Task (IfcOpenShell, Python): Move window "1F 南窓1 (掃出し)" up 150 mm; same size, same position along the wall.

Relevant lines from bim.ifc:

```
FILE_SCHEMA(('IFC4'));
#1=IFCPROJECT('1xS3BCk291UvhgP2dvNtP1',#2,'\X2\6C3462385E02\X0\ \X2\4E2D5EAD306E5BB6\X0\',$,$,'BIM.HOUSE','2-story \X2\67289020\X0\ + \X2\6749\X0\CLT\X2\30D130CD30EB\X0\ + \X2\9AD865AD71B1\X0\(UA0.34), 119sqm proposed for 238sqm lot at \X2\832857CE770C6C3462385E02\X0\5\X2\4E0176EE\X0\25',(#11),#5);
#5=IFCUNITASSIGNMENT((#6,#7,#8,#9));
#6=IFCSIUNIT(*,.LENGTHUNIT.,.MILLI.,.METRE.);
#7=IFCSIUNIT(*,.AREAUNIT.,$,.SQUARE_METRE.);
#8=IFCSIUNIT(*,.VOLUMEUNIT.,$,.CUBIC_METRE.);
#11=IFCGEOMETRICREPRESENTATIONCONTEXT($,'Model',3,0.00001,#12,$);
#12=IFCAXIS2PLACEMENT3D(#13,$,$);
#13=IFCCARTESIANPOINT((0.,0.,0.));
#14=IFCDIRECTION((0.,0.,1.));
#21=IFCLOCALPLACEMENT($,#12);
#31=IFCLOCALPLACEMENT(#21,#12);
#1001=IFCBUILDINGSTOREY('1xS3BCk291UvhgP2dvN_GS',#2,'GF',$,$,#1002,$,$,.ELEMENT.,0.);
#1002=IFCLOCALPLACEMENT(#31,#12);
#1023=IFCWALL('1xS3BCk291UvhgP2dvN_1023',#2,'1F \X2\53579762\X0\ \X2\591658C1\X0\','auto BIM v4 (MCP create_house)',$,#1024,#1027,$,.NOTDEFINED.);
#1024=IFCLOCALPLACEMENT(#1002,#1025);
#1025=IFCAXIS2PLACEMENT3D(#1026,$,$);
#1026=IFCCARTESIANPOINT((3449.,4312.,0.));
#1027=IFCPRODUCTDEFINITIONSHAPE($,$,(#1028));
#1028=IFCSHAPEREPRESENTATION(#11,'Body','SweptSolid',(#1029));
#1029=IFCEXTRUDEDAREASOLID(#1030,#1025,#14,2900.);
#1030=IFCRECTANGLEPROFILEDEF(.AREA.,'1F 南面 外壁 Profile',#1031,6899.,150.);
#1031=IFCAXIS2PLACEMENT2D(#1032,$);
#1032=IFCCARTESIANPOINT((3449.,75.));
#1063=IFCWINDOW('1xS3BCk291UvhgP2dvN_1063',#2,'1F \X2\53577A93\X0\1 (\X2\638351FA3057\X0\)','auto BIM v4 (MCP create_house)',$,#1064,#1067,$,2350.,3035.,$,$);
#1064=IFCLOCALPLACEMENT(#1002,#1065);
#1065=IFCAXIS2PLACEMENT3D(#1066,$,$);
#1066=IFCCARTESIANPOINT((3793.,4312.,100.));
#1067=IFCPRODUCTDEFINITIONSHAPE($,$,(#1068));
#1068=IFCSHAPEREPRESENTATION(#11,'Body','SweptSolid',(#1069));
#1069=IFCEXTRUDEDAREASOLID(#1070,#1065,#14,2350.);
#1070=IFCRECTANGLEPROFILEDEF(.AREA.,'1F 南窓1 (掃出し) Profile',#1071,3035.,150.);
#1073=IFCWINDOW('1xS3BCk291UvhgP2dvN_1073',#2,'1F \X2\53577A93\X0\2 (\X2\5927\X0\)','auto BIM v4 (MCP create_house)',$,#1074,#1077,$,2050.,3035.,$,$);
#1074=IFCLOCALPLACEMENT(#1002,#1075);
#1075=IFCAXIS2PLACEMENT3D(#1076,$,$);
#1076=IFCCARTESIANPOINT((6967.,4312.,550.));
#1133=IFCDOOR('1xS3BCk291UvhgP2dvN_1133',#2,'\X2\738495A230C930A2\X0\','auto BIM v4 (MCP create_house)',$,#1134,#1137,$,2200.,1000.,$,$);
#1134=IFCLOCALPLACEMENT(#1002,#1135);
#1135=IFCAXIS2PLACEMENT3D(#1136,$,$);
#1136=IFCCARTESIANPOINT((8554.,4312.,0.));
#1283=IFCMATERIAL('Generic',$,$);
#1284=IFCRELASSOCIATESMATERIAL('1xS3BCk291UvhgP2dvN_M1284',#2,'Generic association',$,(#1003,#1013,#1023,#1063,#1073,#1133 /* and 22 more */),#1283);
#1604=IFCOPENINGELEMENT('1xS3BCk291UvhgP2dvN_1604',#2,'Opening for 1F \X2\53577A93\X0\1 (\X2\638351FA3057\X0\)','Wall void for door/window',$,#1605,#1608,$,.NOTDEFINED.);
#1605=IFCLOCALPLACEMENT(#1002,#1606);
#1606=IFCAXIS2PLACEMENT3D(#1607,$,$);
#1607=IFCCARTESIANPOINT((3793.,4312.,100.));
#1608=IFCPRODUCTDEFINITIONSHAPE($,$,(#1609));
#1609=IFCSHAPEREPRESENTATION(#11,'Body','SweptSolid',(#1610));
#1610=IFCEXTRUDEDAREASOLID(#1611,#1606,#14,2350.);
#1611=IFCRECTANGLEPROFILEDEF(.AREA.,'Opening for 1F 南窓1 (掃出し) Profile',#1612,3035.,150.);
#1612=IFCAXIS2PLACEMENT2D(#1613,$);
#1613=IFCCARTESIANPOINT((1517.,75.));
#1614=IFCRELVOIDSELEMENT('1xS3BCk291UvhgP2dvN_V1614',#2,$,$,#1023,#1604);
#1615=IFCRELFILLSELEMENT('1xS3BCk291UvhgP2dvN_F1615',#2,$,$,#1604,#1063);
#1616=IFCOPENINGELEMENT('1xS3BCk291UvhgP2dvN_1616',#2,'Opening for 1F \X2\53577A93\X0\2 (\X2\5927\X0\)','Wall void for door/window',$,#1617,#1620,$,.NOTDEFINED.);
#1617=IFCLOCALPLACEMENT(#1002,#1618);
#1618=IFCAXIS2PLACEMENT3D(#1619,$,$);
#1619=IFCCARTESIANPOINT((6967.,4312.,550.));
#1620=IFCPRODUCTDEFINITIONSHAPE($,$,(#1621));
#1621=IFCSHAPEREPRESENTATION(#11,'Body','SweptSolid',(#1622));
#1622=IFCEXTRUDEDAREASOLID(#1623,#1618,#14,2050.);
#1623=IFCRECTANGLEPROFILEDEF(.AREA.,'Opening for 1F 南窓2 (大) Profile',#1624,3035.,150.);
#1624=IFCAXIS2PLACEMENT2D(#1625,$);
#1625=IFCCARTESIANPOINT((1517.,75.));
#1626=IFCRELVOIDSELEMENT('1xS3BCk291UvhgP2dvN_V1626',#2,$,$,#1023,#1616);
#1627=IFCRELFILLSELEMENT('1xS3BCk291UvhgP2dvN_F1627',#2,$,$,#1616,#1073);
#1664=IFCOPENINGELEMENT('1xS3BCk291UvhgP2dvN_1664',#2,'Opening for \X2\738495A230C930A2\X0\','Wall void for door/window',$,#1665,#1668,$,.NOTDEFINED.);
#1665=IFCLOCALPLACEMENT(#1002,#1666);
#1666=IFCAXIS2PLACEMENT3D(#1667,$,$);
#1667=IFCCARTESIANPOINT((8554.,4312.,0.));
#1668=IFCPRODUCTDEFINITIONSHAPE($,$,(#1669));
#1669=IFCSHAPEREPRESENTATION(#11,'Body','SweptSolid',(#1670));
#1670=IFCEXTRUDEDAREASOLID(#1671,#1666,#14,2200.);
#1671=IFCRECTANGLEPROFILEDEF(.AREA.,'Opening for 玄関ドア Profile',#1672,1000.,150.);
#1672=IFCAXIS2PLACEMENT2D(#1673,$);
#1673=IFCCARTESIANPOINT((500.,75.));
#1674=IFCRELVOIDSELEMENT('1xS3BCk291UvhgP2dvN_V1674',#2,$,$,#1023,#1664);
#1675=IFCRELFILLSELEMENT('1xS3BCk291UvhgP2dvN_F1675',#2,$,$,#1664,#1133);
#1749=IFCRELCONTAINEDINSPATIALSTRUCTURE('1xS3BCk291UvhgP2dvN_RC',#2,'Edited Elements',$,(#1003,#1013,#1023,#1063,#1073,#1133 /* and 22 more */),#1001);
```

```python
import numpy as np
import ifcopenshell
import ifcopenshell.api.geometry
import ifcopenshell.util.placement
import ifcopenshell.util.unit

model = ifcopenshell.open("bim.ifc")
unit_scale = ifcopenshell.util.unit.calculate_unit_scale(model)

window = model.by_guid("1xS3BCk291UvhgP2dvN_1063")
opening = window.FillsVoids[0].RelatingOpeningElement
dz = 0.15 / unit_scale

shift = np.array([0.0, 0.0, dz])
# The window is not placed relative to its opening, so move both.
for product in (opening, window):
    matrix = ifcopenshell.util.placement.get_local_placement(product.ObjectPlacement)
    matrix[:3, 3] += shift
    ifcopenshell.api.geometry.edit_object_placement(model, product=product, matrix=matrix, is_si=False)

print(f"moved by {dz * unit_scale:+.3f} m")

model.write("bim-out.ifc")
```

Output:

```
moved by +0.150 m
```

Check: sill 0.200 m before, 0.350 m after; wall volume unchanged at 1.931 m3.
